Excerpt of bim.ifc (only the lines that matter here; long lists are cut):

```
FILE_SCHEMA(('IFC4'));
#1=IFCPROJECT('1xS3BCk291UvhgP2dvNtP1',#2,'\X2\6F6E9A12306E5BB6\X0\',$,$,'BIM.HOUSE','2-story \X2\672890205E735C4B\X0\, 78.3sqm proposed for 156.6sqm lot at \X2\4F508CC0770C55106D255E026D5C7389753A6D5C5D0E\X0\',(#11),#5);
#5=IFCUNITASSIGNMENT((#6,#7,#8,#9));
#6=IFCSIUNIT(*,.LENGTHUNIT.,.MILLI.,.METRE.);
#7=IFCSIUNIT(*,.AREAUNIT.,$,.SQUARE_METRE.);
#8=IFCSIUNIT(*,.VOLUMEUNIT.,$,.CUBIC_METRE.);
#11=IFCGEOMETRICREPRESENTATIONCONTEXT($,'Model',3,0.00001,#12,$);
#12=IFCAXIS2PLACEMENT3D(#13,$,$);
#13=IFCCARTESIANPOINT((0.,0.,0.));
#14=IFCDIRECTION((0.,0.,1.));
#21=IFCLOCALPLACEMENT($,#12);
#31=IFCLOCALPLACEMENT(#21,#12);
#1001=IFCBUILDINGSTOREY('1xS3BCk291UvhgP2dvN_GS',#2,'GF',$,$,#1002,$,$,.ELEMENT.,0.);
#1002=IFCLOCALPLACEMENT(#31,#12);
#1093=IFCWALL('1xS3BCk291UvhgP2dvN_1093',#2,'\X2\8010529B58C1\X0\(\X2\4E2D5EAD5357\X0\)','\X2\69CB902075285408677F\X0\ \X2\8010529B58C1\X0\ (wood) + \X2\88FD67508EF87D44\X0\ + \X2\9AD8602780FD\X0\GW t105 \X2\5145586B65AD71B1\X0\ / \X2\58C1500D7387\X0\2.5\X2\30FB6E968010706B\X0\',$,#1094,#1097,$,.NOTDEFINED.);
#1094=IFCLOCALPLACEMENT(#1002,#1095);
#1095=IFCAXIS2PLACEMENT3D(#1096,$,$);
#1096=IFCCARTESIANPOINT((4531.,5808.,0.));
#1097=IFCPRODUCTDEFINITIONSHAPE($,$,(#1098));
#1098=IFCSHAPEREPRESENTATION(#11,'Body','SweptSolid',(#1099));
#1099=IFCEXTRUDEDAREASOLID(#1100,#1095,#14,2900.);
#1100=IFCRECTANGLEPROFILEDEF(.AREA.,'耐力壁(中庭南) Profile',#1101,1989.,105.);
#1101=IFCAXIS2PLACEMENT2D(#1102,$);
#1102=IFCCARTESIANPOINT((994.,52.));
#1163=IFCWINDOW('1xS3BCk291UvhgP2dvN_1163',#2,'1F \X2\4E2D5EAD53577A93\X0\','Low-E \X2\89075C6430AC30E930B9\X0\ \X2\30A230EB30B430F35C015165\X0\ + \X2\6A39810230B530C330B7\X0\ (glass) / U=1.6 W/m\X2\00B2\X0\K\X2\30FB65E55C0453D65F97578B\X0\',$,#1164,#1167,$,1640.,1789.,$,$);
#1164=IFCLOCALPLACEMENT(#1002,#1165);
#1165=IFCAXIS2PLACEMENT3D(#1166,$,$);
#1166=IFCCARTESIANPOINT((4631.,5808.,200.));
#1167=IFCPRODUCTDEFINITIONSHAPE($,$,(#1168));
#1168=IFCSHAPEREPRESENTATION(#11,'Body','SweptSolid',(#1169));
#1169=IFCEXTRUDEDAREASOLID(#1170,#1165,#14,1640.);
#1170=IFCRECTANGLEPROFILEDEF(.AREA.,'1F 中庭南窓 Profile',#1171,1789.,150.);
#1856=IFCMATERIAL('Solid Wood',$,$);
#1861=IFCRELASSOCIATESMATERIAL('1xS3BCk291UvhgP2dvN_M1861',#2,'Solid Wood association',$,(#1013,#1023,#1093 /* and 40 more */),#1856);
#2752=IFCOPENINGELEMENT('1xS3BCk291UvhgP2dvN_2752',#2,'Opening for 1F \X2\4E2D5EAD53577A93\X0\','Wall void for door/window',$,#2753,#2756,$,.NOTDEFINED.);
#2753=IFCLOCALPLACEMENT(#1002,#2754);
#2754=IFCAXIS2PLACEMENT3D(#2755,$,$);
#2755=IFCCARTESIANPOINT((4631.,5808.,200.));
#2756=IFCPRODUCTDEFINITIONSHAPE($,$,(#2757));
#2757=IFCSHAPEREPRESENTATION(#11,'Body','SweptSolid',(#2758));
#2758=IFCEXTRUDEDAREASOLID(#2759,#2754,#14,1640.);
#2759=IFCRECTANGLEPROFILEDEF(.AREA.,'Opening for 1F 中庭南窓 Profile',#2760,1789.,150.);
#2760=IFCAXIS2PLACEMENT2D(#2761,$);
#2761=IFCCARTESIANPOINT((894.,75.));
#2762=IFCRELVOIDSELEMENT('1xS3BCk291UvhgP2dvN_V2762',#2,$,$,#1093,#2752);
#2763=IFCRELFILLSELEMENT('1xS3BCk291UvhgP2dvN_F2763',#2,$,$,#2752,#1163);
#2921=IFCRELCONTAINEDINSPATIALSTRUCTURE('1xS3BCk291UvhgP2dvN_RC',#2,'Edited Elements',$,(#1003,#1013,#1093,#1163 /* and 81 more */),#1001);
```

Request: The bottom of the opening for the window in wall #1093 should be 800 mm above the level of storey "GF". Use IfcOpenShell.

```python
import numpy as np
import ifcopenshell
import ifcopenshell.api.geometry
import ifcopenshell.geom
import ifcopenshell.util.element
import ifcopenshell.util.placement
import ifcopenshell.util.shape
import ifcopenshell.util.unit

model = ifcopenshell.open("bim.ifc")
unit_scale = ifcopenshell.util.unit.calculate_unit_scale(model)

window = model.by_guid("1xS3BCk291UvhgP2dvN_1163")
opening = window.FillsVoids[0].RelatingOpeningElement
storey = ifcopenshell.util.element.get_container(window, ifc_class="IfcBuildingStorey")
level = ifcopenshell.util.placement.get_local_placement(storey.ObjectPlacement)[2, 3]

# The opening's origin need not be at the sill, so measure its lowest point.
shape = ifcopenshell.geom.create_shape(ifcopenshell.geom.settings(), opening)
bottom = ifcopenshell.util.shape.get_shape_bottom_elevation(shape, shape.geometry) / unit_scale
dz = level + 0.8 / unit_scale - bottom

shift = np.array([0.0, 0.0, dz])
# The window is not placed relative to its opening, so move both.
for product in (opening, window):
    matrix = ifcopenshell.util.placement.get_local_placement(product.ObjectPlacement)
    matrix[:3, 3] += shift
    ifcopenshell.api.geometry.edit_object_placement(model, product=product, matrix=matrix, is_si=False)

print(f"moved by {dz * unit_scale:+.3f} m")

model.write("bim_rev.ifc")
```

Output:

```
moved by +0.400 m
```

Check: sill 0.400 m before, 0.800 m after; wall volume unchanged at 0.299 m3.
